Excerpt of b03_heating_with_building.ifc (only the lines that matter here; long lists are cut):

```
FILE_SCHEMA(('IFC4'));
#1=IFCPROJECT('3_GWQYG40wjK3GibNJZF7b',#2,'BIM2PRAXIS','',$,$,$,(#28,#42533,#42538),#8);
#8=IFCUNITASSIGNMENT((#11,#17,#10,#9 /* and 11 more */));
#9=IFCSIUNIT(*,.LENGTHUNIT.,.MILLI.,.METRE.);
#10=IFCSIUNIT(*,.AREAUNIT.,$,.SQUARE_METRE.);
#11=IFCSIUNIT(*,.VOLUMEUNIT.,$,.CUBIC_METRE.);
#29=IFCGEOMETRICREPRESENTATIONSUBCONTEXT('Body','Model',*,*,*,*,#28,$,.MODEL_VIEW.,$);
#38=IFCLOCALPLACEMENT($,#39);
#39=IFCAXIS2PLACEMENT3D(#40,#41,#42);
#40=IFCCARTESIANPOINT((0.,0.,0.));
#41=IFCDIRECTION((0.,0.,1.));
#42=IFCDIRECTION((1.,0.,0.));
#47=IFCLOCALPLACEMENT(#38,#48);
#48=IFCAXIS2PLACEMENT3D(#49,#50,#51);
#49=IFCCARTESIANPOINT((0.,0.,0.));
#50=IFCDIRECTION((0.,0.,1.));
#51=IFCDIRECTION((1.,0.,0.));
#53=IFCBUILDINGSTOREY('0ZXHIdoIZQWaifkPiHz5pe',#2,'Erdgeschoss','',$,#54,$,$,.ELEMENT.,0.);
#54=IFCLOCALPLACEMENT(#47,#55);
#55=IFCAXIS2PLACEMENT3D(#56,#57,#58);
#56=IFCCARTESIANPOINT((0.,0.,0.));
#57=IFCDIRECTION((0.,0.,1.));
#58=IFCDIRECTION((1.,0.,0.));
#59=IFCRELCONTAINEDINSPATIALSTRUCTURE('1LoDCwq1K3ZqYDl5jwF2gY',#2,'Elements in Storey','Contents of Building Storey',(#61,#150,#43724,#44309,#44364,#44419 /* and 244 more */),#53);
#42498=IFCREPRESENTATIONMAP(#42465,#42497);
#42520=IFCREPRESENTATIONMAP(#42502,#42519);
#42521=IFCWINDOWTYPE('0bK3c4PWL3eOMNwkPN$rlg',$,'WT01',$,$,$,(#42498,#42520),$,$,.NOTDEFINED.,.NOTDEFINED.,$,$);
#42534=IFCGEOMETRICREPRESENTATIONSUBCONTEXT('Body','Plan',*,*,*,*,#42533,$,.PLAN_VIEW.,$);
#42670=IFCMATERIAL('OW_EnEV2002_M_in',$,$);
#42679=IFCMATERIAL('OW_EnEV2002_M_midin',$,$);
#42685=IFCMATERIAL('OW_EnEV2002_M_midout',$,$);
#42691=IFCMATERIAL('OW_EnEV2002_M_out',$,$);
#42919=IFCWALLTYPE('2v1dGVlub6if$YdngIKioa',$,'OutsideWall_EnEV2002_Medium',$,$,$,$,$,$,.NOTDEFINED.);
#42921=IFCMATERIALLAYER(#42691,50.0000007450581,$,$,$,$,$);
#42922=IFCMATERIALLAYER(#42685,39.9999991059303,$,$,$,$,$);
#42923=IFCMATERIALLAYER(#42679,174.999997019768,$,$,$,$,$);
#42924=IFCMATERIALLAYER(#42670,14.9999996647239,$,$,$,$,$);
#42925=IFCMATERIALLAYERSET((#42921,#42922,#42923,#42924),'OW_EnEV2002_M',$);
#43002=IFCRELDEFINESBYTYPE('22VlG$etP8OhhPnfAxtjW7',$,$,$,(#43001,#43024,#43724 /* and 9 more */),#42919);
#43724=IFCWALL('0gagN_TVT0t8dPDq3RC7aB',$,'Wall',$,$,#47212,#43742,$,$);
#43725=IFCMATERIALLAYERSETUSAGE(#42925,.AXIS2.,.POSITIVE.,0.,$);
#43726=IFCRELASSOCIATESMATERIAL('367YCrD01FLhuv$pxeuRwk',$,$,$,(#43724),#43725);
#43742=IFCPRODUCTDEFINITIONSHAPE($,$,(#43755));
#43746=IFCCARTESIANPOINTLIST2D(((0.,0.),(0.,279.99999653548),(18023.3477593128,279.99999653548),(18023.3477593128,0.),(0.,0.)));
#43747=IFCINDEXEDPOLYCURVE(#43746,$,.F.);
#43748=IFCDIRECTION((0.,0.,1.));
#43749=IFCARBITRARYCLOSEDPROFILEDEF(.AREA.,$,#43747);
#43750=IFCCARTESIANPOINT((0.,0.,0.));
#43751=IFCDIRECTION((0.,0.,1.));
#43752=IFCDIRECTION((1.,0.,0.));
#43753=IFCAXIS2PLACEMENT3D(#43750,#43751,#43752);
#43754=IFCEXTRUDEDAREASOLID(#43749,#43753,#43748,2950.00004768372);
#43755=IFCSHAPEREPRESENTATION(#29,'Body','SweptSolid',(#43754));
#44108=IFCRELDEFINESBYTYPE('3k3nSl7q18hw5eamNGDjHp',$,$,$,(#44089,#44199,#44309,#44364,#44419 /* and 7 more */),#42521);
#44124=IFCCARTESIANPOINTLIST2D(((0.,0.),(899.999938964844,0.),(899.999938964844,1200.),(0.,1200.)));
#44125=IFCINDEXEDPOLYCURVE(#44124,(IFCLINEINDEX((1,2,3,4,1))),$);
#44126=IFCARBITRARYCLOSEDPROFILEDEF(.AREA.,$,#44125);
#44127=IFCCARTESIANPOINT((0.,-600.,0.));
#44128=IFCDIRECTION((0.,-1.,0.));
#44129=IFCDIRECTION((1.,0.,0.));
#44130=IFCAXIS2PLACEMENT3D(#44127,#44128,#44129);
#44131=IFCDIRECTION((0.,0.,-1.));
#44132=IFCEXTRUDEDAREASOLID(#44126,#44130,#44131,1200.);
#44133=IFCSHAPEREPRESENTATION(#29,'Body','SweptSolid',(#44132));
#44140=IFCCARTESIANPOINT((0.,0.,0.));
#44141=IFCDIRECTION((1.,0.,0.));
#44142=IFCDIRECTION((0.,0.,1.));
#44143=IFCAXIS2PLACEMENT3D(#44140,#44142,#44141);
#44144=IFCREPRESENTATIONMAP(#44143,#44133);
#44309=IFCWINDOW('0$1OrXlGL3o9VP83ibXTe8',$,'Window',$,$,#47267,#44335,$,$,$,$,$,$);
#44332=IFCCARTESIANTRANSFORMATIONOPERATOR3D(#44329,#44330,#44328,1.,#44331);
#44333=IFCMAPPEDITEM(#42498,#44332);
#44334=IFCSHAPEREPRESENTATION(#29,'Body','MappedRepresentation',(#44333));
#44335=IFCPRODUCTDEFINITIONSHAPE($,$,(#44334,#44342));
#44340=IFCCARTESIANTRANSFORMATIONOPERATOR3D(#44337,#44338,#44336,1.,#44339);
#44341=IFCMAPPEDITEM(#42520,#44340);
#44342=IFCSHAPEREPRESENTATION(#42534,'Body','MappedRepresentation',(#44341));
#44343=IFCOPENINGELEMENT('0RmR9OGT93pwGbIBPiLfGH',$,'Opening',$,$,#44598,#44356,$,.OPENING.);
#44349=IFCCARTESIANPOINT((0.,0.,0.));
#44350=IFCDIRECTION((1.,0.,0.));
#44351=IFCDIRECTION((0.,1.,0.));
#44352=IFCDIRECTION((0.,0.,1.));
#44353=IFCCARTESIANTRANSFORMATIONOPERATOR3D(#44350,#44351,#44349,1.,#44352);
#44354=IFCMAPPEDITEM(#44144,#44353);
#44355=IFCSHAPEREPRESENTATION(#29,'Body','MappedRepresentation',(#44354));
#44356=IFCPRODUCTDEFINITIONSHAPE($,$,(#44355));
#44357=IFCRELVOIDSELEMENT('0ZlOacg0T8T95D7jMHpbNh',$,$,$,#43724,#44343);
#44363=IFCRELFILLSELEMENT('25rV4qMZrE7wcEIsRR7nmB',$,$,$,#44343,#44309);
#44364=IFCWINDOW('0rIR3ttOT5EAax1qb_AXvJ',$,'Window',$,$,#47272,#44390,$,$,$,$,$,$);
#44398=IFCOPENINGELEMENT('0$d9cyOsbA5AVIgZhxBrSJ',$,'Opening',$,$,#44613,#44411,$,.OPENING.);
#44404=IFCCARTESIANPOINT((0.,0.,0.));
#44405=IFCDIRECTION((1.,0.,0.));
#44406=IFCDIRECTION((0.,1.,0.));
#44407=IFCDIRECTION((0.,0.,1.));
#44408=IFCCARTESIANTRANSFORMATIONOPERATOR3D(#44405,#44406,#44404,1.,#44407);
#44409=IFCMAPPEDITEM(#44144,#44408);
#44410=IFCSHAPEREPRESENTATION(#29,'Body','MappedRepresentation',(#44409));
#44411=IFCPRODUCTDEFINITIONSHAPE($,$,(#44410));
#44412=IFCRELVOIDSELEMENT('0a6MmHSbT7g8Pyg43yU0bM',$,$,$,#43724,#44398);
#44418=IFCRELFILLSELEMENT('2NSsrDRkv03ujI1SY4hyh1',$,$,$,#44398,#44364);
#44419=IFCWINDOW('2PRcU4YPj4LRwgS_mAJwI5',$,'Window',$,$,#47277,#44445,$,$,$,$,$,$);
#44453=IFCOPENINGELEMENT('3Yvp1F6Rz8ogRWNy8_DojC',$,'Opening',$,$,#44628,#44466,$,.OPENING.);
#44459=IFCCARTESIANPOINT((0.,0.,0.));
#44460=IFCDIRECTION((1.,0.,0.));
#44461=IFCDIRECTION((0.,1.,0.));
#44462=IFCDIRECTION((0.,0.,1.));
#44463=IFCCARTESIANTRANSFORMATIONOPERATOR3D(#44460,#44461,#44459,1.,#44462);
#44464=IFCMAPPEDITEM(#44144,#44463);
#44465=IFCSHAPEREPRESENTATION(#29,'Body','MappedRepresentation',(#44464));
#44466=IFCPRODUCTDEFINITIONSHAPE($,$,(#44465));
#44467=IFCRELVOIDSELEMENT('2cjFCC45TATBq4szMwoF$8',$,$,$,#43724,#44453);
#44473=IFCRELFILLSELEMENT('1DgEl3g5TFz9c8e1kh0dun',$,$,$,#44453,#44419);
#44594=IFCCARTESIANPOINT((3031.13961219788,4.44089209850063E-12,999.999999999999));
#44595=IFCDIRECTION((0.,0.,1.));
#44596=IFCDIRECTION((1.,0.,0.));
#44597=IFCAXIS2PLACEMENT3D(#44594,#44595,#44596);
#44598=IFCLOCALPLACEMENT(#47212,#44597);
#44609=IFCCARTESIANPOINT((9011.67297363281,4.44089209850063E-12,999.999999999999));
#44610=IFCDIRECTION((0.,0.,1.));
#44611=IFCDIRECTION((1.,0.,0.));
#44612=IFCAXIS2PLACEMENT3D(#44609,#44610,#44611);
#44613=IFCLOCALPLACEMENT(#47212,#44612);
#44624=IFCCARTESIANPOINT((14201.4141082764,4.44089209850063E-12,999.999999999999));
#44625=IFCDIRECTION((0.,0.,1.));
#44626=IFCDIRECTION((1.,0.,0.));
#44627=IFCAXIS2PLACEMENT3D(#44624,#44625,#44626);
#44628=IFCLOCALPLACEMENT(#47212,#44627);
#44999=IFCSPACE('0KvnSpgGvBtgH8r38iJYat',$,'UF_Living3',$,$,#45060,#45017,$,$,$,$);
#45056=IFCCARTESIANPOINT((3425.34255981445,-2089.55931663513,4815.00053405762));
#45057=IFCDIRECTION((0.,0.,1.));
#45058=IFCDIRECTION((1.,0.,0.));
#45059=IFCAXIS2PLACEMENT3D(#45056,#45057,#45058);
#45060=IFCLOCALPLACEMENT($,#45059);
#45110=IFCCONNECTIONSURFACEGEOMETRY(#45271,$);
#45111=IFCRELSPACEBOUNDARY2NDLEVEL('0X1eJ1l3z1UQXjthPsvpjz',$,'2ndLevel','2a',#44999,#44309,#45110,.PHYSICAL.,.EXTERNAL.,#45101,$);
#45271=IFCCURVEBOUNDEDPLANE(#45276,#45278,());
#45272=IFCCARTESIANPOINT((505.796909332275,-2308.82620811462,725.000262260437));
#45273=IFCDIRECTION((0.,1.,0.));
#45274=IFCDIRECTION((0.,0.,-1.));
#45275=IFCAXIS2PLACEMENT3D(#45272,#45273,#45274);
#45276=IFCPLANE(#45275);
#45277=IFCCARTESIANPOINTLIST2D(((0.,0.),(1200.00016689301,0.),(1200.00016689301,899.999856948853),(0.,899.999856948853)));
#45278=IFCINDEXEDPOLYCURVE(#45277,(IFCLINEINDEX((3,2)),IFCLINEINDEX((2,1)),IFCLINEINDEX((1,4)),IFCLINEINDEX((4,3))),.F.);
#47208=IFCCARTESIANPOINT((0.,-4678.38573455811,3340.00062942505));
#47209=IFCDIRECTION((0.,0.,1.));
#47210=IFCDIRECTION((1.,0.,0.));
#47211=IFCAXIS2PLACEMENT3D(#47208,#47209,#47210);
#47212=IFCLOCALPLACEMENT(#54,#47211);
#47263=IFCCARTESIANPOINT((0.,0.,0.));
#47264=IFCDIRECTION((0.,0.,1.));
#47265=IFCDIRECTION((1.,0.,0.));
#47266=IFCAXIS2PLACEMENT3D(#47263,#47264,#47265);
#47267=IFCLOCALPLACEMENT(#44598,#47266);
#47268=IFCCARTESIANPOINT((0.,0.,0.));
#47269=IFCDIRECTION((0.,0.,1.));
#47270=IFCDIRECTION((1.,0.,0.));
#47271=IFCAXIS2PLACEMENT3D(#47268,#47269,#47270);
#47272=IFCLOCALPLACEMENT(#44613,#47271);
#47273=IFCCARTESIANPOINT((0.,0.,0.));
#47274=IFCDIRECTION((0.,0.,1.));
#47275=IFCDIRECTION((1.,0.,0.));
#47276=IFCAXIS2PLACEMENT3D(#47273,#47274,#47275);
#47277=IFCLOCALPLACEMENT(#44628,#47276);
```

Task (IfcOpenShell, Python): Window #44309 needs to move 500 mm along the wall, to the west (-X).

```python
import numpy as np
import ifcopenshell
import ifcopenshell.api.geometry
import ifcopenshell.util.placement

model = ifcopenshell.open("b03_heating_with_building.ifc")

window = model.by_id(44309)
opening = window.FillsVoids[0].RelatingOpeningElement
wall = opening.VoidsElements[0].RelatingBuildingElement

wall_matrix = ifcopenshell.util.placement.get_local_placement(wall.ObjectPlacement)
shift = wall_matrix[:3, 0] * -500.0
before = ifcopenshell.util.placement.get_local_placement(window.ObjectPlacement)[:3, 3].copy()

# The window is placed relative to its opening, so it follows when the opening moves.
matrix = ifcopenshell.util.placement.get_local_placement(opening.ObjectPlacement)
matrix[:3, 3] += shift
ifcopenshell.api.geometry.edit_object_placement(
    model, product=opening, matrix=matrix, is_si=False, should_transform_children=True
)

# Space boundary surfaces are stored in each space's coordinates; move them too.
for rel in window.ProvidesBoundaries:
    if not rel.ConnectionGeometry:
        continue
    surface = rel.ConnectionGeometry.SurfaceOnRelatingElement.BasisSurface
    space_matrix = ifcopenshell.util.placement.get_local_placement(rel.RelatingSpace.ObjectPlacement)
    point = np.array(surface.Position.Location.Coordinates) + space_matrix[:3, :3].T @ shift
    surface.Position = model.createIfcAxis2Placement3D(
        model.createIfcCartesianPoint(point.tolist()), surface.Position.Axis, surface.Position.RefDirection
    )

after = ifcopenshell.util.placement.get_local_placement(window.ObjectPlacement)[:3, 3]
print("window moved by", (after - before).round(3) + 0.0)

model.write("b03_heating_with_building_updated.ifc")
```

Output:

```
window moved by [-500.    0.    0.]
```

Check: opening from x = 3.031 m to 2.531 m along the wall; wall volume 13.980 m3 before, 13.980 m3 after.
